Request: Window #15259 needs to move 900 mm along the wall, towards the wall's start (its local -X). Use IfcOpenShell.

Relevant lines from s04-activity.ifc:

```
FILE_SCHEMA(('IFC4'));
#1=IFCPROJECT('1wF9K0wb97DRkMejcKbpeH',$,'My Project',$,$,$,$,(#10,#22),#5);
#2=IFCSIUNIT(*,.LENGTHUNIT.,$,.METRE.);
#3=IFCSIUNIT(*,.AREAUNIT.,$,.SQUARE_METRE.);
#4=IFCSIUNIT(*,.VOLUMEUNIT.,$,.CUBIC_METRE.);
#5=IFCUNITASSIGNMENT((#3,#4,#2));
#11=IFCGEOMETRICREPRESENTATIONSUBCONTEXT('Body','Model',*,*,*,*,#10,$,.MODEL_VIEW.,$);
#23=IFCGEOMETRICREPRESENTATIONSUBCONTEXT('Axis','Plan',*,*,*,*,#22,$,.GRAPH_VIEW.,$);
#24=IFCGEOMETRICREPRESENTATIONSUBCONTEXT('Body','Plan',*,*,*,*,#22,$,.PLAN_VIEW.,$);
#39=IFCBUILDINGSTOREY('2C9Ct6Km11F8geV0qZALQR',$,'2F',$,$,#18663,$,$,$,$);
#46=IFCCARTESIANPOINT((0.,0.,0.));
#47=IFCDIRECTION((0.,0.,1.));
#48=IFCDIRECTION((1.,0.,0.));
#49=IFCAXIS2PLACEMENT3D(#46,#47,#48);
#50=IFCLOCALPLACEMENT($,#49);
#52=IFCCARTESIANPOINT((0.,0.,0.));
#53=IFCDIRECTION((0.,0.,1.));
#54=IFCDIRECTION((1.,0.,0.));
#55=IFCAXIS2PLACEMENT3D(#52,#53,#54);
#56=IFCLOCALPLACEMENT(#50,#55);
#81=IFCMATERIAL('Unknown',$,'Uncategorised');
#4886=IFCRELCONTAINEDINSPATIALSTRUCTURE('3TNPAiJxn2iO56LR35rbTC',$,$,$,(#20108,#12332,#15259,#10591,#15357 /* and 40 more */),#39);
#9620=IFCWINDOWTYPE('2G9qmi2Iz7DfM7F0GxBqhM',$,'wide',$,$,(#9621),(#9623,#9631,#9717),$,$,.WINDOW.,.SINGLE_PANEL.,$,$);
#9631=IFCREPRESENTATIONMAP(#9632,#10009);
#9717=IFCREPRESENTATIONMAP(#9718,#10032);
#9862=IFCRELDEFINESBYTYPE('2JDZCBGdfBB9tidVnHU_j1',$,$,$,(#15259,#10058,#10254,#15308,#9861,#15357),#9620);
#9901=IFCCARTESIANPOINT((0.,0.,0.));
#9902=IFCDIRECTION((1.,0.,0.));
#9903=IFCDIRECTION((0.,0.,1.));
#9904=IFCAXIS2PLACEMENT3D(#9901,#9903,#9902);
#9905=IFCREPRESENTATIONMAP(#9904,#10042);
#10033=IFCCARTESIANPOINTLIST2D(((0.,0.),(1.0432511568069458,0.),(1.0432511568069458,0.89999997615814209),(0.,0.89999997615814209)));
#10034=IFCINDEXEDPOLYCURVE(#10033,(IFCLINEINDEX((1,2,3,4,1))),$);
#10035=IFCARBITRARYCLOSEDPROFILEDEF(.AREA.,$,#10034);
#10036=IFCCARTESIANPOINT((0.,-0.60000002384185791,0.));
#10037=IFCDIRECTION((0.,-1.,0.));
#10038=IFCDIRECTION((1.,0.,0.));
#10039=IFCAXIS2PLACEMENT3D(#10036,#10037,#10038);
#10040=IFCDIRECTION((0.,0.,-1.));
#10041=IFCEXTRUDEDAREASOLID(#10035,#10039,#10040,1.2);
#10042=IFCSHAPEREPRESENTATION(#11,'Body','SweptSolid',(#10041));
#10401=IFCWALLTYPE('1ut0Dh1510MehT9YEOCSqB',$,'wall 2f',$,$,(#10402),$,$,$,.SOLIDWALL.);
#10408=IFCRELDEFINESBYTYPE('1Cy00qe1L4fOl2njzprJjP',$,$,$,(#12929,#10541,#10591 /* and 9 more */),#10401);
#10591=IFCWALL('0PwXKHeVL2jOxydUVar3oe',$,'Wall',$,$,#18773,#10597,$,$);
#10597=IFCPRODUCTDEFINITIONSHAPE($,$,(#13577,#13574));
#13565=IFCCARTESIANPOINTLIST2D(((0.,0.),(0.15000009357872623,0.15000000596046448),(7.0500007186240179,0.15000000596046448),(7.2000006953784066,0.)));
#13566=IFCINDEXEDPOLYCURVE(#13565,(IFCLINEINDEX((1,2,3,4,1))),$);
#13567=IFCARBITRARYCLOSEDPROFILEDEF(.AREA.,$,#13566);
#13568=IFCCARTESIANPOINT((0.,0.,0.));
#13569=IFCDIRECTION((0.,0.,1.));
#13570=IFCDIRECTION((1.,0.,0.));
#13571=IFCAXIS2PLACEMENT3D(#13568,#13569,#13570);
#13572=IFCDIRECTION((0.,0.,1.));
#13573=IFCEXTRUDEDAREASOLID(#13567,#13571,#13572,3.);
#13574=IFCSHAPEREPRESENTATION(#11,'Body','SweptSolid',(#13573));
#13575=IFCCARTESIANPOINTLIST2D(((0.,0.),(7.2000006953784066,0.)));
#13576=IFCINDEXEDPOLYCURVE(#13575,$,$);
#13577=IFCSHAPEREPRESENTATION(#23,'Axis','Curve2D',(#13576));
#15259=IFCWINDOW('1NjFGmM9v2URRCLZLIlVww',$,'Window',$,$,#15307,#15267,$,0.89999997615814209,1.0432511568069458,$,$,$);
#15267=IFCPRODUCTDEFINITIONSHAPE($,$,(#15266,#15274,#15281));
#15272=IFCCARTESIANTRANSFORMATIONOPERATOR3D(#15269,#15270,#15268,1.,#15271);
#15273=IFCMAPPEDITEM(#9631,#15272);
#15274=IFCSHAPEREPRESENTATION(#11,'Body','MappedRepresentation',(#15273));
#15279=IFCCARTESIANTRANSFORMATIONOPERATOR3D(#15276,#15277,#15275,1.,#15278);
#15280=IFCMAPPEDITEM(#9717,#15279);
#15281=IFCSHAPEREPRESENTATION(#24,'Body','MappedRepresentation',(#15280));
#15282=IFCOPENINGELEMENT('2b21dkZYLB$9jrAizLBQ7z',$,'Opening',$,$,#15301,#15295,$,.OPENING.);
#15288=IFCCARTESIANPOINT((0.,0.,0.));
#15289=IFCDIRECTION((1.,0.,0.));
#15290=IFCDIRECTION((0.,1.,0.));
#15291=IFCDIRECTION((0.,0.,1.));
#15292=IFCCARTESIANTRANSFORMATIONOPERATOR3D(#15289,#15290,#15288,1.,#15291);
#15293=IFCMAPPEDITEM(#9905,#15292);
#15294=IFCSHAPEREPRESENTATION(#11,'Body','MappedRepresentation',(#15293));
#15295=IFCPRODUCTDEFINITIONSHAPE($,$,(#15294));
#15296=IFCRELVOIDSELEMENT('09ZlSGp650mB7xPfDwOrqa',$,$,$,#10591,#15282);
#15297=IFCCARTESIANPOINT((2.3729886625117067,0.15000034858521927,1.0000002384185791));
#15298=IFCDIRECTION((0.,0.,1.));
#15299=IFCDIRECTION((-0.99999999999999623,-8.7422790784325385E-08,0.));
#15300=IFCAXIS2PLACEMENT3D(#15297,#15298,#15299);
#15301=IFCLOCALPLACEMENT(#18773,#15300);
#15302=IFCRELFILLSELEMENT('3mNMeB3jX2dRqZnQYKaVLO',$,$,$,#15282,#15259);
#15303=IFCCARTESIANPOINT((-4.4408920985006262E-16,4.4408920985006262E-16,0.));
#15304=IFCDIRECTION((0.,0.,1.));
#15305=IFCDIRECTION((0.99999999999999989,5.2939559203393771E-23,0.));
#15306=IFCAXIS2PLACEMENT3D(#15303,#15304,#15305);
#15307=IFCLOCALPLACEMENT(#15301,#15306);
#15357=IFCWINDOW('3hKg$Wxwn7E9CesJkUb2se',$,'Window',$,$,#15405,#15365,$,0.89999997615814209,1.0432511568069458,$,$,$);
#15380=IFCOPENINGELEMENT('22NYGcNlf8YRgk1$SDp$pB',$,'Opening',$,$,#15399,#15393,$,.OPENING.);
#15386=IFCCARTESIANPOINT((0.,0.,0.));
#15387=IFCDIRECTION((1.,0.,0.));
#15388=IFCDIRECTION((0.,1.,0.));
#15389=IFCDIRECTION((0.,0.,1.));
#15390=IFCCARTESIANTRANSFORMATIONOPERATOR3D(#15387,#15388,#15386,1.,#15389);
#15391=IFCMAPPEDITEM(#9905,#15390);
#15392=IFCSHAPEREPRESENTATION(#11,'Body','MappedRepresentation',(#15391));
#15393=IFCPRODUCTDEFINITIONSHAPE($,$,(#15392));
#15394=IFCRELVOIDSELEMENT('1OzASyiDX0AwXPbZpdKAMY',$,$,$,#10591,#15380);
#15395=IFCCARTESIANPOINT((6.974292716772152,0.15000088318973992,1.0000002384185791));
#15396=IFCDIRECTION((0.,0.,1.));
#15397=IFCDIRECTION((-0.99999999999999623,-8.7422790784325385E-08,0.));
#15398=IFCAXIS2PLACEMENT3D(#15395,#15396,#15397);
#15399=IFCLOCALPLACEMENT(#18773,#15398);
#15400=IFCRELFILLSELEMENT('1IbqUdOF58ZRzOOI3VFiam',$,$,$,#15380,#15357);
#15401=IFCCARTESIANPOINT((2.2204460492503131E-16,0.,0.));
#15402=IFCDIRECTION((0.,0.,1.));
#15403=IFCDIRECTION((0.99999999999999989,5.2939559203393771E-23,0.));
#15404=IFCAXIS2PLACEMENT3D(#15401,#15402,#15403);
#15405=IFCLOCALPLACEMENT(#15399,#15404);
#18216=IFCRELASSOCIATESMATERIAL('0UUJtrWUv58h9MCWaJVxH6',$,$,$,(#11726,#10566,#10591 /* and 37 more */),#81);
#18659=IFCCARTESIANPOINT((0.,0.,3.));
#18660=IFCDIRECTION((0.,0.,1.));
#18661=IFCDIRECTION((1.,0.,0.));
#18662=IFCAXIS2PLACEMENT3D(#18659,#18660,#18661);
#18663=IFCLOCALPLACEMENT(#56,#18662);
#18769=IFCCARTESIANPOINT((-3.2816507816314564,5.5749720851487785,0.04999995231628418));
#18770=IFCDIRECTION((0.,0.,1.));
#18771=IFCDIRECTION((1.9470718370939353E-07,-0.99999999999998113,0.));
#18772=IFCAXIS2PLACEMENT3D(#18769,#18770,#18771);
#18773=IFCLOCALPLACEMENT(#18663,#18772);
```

```python
import ifcopenshell
import ifcopenshell.api.geometry
import ifcopenshell.util.placement

model = ifcopenshell.open("s04-activity.ifc")

window = model.by_guid("1NjFGmM9v2URRCLZLIlVww")
opening = window.FillsVoids[0].RelatingOpeningElement
wall = opening.VoidsElements[0].RelatingBuildingElement

wall_matrix = ifcopenshell.util.placement.get_local_placement(wall.ObjectPlacement)
shift = wall_matrix[:3, 0] * -0.9
before = ifcopenshell.util.placement.get_local_placement(window.ObjectPlacement)[:3, 3].copy()

# The window is placed relative to its opening, so it follows when the opening moves.
matrix = ifcopenshell.util.placement.get_local_placement(opening.ObjectPlacement)
matrix[:3, 3] += shift
ifcopenshell.api.geometry.edit_object_placement(
    model, product=opening, matrix=matrix, is_si=False, should_transform_children=True
)

after = ifcopenshell.util.placement.get_local_placement(window.ObjectPlacement)[:3, 3]
print("window moved by", (after - before).round(3) + 0.0)

model.write("s04-activity_updated.ifc")
```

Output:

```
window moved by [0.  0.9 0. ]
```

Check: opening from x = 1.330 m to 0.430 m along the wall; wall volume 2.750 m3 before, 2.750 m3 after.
